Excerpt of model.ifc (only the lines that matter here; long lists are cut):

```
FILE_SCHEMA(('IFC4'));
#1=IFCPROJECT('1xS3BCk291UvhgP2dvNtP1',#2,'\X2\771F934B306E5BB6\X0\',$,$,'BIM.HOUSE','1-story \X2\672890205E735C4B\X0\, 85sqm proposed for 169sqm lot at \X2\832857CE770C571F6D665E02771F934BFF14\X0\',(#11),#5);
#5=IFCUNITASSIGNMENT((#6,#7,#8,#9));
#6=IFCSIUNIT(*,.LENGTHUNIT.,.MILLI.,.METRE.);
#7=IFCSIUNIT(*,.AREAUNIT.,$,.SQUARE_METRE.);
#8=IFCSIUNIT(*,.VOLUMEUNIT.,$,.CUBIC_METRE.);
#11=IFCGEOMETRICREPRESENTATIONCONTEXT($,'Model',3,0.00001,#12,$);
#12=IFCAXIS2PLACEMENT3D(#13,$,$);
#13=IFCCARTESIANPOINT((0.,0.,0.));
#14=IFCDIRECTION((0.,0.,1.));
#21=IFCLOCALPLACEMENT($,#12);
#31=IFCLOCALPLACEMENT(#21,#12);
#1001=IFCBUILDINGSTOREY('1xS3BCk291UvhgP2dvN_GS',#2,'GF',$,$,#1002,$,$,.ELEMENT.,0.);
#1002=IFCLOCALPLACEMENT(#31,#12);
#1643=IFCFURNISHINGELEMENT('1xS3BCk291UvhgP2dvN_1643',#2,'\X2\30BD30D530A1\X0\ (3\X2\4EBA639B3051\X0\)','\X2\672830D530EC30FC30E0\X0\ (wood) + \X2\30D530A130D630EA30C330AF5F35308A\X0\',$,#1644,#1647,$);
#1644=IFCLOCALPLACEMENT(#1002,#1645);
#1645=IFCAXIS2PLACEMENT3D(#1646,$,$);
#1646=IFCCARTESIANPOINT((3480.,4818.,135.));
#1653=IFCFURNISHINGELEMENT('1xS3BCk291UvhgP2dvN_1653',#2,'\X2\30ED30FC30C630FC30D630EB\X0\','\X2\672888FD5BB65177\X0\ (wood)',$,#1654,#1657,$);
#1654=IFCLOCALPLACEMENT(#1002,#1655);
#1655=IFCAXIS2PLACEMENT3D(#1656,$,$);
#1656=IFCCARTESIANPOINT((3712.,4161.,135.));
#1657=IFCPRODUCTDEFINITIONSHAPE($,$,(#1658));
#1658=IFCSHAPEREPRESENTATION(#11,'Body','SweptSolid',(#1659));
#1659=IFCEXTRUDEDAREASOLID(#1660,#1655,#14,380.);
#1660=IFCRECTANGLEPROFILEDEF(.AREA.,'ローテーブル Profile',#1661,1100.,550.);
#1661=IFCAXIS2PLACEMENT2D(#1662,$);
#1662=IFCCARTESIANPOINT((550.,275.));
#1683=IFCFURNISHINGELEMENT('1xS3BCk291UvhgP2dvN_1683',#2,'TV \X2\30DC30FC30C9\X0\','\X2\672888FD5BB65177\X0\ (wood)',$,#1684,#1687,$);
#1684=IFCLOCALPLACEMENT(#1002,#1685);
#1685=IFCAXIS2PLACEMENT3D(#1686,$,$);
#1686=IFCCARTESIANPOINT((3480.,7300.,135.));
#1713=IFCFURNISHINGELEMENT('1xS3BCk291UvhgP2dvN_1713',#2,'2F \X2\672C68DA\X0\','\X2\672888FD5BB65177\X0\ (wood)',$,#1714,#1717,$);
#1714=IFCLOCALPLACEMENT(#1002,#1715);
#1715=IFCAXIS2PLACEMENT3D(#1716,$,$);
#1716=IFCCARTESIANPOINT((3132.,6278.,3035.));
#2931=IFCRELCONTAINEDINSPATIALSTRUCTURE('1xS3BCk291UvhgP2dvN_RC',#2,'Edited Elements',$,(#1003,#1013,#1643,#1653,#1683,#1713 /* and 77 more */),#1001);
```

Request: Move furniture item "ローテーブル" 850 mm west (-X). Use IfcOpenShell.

```python
import ifcopenshell
import ifcopenshell.api.geometry
import ifcopenshell.util.placement
import ifcopenshell.util.unit

model = ifcopenshell.open("model.ifc")
unit_scale = ifcopenshell.util.unit.calculate_unit_scale(model)

item = model.by_guid("1xS3BCk291UvhgP2dvN_1653")
matrix = ifcopenshell.util.placement.get_local_placement(item.ObjectPlacement)
matrix[0, 3] -= 0.85 / unit_scale
ifcopenshell.api.geometry.edit_object_placement(model, product=item, matrix=matrix, is_si=False)

print(ifcopenshell.util.placement.get_local_placement(item.ObjectPlacement).round(3) + 0.0)

model.write("model-out.ifc")
```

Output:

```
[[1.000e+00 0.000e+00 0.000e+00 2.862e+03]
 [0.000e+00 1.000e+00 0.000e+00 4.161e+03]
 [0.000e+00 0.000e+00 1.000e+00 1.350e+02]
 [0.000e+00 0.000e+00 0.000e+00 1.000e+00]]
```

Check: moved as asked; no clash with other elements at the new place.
